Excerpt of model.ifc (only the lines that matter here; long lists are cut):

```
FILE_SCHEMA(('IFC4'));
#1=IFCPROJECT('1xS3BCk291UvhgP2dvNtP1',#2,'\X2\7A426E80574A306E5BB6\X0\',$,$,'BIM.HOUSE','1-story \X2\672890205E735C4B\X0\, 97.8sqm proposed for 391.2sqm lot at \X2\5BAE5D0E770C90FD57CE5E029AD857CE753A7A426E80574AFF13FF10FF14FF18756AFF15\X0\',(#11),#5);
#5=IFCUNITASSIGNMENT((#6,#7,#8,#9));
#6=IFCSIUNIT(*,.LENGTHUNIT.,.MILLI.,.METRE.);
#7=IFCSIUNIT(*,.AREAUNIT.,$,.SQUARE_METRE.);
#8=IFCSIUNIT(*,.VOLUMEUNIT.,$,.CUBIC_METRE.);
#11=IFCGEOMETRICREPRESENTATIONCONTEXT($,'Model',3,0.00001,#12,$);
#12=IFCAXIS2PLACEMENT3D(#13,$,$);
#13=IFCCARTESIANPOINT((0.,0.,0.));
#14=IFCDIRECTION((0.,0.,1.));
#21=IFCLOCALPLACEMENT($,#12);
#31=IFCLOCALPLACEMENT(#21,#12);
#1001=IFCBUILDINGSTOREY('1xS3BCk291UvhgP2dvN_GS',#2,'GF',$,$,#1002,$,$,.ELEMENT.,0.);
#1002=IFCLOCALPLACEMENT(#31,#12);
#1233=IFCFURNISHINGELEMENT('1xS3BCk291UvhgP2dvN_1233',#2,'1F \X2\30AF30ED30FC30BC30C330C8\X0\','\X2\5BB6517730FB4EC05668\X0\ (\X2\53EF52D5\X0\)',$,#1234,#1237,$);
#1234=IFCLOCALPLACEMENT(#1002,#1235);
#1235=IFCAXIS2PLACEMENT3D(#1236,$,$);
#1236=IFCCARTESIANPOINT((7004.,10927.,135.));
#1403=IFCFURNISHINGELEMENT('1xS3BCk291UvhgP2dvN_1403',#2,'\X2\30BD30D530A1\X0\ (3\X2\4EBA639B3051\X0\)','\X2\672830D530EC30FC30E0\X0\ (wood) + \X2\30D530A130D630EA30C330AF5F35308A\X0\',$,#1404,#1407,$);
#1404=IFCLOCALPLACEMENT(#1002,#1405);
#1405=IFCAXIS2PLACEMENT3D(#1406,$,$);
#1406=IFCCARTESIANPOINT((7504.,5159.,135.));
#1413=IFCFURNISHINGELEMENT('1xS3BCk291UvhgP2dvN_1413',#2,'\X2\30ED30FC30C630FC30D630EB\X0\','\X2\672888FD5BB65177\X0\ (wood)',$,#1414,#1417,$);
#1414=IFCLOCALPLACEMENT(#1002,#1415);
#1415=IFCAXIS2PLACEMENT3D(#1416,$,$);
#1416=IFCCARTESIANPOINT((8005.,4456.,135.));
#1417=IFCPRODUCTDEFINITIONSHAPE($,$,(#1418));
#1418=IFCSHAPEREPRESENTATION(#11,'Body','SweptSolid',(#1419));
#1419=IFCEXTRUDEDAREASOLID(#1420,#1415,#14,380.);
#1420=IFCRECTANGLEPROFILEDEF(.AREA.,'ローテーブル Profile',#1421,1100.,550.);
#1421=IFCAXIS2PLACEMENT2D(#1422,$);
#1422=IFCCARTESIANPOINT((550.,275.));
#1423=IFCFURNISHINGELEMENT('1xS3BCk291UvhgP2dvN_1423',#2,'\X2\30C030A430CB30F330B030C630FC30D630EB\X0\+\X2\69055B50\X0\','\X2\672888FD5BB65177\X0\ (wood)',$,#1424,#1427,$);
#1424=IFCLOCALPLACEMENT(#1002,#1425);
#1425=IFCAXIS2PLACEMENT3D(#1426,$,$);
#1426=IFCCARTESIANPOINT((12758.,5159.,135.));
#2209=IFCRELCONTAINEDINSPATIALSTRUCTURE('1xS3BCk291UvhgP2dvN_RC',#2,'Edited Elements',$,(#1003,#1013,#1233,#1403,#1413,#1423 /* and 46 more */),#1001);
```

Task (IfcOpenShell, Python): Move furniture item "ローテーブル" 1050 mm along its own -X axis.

```python
import ifcopenshell
import ifcopenshell.api.geometry
import ifcopenshell.util.placement

model = ifcopenshell.open("model.ifc")

item = model.by_id(1413)
matrix = ifcopenshell.util.placement.get_local_placement(item.ObjectPlacement)
matrix[:3, 3] -= matrix[:3, 0] * 1050.0
ifcopenshell.api.geometry.edit_object_placement(model, product=item, matrix=matrix, is_si=False)

print(ifcopenshell.util.placement.get_local_placement(item.ObjectPlacement).round(3) + 0.0)

model.write("model-out.ifc")
```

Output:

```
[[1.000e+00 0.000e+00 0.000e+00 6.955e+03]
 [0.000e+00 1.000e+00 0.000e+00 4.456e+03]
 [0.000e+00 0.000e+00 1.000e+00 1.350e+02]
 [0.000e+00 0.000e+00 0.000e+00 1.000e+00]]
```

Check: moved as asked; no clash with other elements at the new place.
